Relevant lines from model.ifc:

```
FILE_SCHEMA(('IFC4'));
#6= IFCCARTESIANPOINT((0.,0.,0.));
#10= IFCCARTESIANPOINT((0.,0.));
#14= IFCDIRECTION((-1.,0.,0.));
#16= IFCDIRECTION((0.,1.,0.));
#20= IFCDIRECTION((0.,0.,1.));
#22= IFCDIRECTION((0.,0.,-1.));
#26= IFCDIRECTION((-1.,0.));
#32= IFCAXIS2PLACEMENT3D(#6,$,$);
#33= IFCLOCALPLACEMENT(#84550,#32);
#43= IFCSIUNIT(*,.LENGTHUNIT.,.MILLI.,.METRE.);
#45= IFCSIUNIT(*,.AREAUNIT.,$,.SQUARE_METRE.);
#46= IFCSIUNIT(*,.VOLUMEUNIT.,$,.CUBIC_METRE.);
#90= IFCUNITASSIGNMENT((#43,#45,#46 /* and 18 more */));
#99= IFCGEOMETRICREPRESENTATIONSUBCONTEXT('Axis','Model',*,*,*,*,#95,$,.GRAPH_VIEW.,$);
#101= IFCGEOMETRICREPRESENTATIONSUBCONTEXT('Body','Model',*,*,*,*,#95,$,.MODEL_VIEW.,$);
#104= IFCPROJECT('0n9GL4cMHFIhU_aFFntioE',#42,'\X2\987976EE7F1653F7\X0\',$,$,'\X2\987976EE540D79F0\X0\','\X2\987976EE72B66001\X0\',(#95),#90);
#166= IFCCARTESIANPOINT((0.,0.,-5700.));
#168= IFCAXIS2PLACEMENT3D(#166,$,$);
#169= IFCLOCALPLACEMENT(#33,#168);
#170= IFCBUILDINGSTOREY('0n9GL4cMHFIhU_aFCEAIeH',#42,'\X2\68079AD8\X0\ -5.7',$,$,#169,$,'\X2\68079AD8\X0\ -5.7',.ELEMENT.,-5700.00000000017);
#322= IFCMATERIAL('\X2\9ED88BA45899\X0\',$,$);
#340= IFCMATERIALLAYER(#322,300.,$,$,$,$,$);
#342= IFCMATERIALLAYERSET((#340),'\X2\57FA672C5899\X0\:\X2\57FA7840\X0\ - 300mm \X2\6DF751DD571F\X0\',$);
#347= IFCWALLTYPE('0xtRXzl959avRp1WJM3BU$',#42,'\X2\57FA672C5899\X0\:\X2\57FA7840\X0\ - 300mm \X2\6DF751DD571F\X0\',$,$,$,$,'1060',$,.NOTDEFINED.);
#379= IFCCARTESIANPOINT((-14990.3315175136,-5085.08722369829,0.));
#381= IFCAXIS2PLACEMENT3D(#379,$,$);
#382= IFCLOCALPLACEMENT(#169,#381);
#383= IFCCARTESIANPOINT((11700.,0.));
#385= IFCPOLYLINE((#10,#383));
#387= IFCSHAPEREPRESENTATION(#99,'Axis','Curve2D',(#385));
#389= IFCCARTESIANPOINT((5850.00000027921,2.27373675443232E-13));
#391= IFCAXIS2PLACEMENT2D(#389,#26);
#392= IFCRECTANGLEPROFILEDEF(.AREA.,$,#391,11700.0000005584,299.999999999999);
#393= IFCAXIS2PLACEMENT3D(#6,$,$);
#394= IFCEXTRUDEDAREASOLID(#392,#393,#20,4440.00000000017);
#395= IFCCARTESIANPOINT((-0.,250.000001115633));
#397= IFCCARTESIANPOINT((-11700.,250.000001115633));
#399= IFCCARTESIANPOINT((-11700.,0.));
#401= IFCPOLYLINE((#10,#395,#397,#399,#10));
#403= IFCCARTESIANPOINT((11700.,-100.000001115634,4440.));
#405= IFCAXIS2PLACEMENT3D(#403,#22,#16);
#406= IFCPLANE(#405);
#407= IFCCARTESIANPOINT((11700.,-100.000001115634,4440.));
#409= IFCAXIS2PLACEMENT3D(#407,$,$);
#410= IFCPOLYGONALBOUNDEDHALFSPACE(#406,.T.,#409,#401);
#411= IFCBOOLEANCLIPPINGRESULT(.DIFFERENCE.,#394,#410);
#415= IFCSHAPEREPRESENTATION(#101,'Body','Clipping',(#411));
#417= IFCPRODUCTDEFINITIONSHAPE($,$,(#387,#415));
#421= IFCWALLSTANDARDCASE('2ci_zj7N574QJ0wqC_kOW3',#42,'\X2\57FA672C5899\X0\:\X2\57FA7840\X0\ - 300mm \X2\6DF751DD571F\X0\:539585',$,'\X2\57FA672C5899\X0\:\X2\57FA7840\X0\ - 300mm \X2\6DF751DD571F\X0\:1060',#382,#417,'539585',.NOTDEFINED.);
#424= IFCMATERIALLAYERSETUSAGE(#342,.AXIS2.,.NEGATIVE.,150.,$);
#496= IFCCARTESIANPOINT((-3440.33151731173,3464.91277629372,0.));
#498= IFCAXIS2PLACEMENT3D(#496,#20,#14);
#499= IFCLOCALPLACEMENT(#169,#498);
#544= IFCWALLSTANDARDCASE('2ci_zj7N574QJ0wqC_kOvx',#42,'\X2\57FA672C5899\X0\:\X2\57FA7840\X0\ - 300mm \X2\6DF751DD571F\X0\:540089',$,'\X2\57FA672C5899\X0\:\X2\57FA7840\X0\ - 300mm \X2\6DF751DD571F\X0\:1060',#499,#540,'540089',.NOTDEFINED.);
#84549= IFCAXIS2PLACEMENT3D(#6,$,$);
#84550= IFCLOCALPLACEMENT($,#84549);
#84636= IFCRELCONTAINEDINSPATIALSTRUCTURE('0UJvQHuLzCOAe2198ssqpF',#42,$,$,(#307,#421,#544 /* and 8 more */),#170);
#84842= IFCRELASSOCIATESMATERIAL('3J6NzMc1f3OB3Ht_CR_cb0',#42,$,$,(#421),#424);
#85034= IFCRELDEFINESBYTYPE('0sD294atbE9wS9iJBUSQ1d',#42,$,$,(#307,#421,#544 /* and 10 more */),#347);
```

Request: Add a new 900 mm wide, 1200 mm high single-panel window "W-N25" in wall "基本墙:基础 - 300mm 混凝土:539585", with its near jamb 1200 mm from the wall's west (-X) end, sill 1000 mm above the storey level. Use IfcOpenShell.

```python
import numpy as np
import ifcopenshell
import ifcopenshell.api.feature
import ifcopenshell.api.geometry
import ifcopenshell.api.root
import ifcopenshell.api.spatial
import ifcopenshell.geom
import ifcopenshell.util.element
import ifcopenshell.util.placement
import ifcopenshell.util.representation
import ifcopenshell.util.shape
import ifcopenshell.util.unit

model = ifcopenshell.open("model.ifc")
unit_scale = ifcopenshell.util.unit.calculate_unit_scale(model)
settings = ifcopenshell.geom.settings()


def volume(element):
    """Net volume in cubic metres, openings subtracted."""
    shape = ifcopenshell.geom.create_shape(settings, element)
    return ifcopenshell.util.shape.get_volume(shape.geometry)


wall = model.by_guid("2ci_zj7N574QJ0wqC_kOW3")
storey = ifcopenshell.util.element.get_container(wall, ifc_class="IfcBuildingStorey")
context = ifcopenshell.util.representation.get_context(model, "Model", "Body", "MODEL_VIEW")
before = volume(wall)

width, height, from_end, sill = 0.9, 1.2, 1.2, 1  # metres

# The wall runs along its own X axis, and the end named is its -X end.
wall_shape = ifcopenshell.geom.create_shape(settings, wall)
x, y, z = ifcopenshell.util.shape.get_vertices(wall_shape.geometry).T
start = x.min() + from_end
face, thickness = float(y.min()), float(y.max() - y.min())
wall_matrix = ifcopenshell.util.placement.get_local_placement(wall.ObjectPlacement)
level = ifcopenshell.util.placement.get_local_placement(storey.ObjectPlacement)[2, 3]


def in_wall(x, y):
    """Placement at x, y metres in the wall's axes, at sill height."""
    matrix = wall_matrix.copy()
    matrix[:, 3] = wall_matrix @ np.array([x / unit_scale, y / unit_scale, 0.0, 1.0])
    matrix[2, 3] = level + sill / unit_scale
    return matrix


# Opening: a box that overshoots both wall faces by 50 mm.
opening = ifcopenshell.api.root.create_entity(model, ifc_class="IfcOpeningElement", predefined_type="OPENING")
box = ifcopenshell.api.geometry.add_wall_representation(
    model, context=context, length=width, height=height, thickness=thickness + 0.1
)
ifcopenshell.api.geometry.assign_representation(model, product=opening, representation=box)
ifcopenshell.api.geometry.edit_object_placement(model, product=opening, matrix=in_wall(start, face - 0.05), is_si=False)
ifcopenshell.api.feature.add_feature(model, feature=opening, element=wall)

window = ifcopenshell.api.root.create_entity(model, ifc_class="IfcWindow", name="W-N25", predefined_type="WINDOW")
window.OverallWidth, window.OverallHeight = width / unit_scale, height / unit_scale
window.PartitioningType = "SINGLE_PANEL"
body = ifcopenshell.api.geometry.add_window_representation(
    model,
    context=context,
    overall_width=window.OverallWidth,
    overall_height=window.OverallHeight,
    partition_type="SINGLE_PANEL",
)
ifcopenshell.api.geometry.assign_representation(model, product=window, representation=body)
ifcopenshell.api.spatial.assign_container(model, products=[window], relating_structure=storey)
ifcopenshell.api.feature.add_filling(model, opening=opening, element=window)

# Centre the window in the wall's thickness.
ifcopenshell.api.geometry.edit_object_placement(model, product=window, matrix=in_wall(start, face), is_si=False)
window_shape = ifcopenshell.geom.create_shape(settings, window)
depth = ifcopenshell.util.shape.get_vertices(window_shape.geometry)[:, 1]
offset = face + thickness / 2 - (depth.min() + depth.max()) / 2
ifcopenshell.api.geometry.edit_object_placement(model, product=window, matrix=in_wall(start, offset), is_si=False)

after = volume(wall)

print(f"wall volume {before:.3f} -> {after:.3f} m3")

model.write("model-out.ifc")
```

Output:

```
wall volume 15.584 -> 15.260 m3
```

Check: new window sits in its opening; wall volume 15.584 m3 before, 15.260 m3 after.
